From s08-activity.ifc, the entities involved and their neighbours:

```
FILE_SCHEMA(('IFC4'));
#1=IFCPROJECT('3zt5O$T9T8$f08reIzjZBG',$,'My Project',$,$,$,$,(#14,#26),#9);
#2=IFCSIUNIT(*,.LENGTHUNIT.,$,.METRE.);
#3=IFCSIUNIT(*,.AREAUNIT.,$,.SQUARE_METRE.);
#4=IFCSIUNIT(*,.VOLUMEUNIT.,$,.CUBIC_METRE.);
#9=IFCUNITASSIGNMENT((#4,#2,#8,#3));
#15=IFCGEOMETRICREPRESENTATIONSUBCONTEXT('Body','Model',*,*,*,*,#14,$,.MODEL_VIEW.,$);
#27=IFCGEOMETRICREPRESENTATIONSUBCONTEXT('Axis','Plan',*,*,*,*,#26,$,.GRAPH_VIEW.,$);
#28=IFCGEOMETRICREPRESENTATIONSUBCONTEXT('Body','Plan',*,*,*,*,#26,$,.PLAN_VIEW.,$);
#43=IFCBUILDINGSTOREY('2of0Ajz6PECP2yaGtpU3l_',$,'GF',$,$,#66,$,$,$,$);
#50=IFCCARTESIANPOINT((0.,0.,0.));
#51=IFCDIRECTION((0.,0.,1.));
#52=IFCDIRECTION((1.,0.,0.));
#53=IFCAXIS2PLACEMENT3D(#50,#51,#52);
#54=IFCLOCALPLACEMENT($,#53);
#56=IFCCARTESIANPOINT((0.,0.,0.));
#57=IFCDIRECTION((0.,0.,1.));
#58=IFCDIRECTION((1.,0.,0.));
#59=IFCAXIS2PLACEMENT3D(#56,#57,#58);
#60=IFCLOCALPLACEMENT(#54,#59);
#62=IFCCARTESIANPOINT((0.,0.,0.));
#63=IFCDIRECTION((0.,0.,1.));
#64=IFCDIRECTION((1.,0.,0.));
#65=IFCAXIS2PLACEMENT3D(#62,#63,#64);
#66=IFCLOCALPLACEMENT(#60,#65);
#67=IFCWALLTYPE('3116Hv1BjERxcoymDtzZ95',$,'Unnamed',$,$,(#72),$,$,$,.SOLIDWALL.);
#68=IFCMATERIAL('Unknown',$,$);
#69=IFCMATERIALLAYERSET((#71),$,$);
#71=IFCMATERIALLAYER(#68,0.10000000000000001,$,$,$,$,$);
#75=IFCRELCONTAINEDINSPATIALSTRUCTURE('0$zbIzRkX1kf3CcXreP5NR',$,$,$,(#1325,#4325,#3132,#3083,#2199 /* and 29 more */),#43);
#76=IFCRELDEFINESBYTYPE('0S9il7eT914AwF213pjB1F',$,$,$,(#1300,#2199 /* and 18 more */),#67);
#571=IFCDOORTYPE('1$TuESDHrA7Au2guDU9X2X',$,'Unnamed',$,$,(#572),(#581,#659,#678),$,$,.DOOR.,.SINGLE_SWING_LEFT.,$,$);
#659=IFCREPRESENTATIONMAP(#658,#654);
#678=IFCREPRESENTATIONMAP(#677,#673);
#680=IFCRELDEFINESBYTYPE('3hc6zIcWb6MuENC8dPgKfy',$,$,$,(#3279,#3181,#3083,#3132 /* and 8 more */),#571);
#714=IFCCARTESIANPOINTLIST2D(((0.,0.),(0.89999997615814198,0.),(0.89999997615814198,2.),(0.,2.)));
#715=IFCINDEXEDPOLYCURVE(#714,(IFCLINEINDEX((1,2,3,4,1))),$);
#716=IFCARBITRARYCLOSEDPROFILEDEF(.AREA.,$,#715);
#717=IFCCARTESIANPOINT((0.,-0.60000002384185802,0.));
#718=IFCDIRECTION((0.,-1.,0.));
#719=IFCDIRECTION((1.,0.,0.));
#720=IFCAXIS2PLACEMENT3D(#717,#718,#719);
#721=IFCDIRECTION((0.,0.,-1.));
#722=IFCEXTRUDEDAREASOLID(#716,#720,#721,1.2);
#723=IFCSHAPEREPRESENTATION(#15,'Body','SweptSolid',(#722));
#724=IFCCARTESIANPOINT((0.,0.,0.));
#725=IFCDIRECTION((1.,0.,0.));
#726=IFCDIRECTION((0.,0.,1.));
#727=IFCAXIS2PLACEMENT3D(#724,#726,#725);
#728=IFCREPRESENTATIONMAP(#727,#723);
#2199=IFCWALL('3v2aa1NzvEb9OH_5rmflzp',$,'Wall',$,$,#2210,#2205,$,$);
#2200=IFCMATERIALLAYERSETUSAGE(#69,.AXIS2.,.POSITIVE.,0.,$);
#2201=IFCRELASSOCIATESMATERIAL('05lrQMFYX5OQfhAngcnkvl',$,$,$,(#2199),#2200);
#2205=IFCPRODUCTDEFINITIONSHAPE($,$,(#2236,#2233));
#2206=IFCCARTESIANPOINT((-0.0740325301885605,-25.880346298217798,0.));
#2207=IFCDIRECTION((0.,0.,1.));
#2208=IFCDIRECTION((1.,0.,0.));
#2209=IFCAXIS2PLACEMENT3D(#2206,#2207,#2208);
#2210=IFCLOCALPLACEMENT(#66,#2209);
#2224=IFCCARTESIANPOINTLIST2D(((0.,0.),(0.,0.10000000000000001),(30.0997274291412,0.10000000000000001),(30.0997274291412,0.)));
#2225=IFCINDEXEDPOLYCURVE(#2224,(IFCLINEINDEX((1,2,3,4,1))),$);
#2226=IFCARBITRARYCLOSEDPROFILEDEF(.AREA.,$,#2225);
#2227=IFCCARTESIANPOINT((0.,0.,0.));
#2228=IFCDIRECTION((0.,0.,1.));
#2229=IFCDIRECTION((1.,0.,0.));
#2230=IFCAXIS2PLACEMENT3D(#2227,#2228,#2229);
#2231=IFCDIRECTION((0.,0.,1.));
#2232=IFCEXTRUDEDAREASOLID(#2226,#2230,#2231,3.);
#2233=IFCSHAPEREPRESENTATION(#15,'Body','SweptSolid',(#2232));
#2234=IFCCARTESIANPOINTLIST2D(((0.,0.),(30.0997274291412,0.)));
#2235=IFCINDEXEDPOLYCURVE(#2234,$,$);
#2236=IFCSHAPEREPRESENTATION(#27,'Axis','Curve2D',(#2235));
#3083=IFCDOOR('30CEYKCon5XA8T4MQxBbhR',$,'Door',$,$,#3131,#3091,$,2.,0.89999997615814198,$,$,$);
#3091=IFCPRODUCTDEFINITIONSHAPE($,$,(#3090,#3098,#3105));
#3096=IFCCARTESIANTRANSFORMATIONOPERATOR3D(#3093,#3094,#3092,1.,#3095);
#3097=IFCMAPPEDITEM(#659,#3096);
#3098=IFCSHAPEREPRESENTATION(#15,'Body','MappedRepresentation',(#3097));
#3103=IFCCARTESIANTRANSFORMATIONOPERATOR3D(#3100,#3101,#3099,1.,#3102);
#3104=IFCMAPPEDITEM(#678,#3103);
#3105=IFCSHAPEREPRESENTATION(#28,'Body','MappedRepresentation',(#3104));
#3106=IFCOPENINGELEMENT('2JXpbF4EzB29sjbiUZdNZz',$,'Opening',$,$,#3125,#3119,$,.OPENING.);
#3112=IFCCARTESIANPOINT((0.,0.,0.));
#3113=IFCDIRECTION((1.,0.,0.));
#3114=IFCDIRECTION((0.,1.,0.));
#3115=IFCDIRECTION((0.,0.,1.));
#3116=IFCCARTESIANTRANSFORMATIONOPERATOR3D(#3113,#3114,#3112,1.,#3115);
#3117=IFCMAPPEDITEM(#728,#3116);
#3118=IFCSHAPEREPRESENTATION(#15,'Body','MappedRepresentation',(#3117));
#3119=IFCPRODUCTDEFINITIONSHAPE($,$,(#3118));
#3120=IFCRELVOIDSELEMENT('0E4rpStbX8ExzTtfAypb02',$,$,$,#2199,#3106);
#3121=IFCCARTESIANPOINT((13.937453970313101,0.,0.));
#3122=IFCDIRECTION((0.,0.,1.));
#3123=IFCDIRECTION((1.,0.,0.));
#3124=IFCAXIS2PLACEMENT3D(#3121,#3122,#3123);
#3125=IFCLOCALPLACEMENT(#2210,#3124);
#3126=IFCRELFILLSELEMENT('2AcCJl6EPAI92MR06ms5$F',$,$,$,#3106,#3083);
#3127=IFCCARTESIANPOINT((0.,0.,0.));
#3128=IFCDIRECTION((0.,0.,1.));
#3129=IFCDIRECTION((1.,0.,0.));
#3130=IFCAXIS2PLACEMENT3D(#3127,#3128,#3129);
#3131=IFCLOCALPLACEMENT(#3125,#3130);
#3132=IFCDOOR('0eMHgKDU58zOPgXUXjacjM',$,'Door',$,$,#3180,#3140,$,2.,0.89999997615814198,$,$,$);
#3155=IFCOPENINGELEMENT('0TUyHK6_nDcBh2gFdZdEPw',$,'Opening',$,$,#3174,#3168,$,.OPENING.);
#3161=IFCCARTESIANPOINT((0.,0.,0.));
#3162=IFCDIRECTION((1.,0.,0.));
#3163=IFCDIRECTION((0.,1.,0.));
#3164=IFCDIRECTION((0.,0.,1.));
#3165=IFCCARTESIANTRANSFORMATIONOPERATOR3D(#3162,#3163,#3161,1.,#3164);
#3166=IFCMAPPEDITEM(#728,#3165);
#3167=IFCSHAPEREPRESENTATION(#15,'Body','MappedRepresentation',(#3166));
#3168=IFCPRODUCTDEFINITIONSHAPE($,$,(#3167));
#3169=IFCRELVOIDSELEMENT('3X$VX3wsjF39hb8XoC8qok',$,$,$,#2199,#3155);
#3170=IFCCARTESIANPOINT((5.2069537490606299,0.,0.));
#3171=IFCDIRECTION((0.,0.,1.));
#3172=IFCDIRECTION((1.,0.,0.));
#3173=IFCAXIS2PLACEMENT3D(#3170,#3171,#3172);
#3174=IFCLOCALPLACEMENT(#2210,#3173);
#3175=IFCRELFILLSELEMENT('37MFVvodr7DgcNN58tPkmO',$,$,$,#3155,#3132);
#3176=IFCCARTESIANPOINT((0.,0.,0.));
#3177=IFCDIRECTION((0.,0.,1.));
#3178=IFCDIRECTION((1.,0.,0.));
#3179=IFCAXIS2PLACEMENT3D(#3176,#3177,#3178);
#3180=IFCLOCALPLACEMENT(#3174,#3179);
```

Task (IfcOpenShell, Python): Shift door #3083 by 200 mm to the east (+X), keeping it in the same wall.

```python
import ifcopenshell
import ifcopenshell.api.geometry
import ifcopenshell.util.placement

model = ifcopenshell.open("s08-activity.ifc")

door = model.by_guid("30CEYKCon5XA8T4MQxBbhR")
opening = door.FillsVoids[0].RelatingOpeningElement
wall = opening.VoidsElements[0].RelatingBuildingElement

wall_matrix = ifcopenshell.util.placement.get_local_placement(wall.ObjectPlacement)
shift = wall_matrix[:3, 0] * 0.2
before = ifcopenshell.util.placement.get_local_placement(door.ObjectPlacement)[:3, 3].copy()

# The door is placed relative to its opening, so it follows when the opening moves.
matrix = ifcopenshell.util.placement.get_local_placement(opening.ObjectPlacement)
matrix[:3, 3] += shift
ifcopenshell.api.geometry.edit_object_placement(
    model, product=opening, matrix=matrix, is_si=False, should_transform_children=True
)

after = ifcopenshell.util.placement.get_local_placement(door.ObjectPlacement)[:3, 3]
print("door moved by", (after - before).round(3) + 0.0)

model.write("s08-activity_updated.ifc")
```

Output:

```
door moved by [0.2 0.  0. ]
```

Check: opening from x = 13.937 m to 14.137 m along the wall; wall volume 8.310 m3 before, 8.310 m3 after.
